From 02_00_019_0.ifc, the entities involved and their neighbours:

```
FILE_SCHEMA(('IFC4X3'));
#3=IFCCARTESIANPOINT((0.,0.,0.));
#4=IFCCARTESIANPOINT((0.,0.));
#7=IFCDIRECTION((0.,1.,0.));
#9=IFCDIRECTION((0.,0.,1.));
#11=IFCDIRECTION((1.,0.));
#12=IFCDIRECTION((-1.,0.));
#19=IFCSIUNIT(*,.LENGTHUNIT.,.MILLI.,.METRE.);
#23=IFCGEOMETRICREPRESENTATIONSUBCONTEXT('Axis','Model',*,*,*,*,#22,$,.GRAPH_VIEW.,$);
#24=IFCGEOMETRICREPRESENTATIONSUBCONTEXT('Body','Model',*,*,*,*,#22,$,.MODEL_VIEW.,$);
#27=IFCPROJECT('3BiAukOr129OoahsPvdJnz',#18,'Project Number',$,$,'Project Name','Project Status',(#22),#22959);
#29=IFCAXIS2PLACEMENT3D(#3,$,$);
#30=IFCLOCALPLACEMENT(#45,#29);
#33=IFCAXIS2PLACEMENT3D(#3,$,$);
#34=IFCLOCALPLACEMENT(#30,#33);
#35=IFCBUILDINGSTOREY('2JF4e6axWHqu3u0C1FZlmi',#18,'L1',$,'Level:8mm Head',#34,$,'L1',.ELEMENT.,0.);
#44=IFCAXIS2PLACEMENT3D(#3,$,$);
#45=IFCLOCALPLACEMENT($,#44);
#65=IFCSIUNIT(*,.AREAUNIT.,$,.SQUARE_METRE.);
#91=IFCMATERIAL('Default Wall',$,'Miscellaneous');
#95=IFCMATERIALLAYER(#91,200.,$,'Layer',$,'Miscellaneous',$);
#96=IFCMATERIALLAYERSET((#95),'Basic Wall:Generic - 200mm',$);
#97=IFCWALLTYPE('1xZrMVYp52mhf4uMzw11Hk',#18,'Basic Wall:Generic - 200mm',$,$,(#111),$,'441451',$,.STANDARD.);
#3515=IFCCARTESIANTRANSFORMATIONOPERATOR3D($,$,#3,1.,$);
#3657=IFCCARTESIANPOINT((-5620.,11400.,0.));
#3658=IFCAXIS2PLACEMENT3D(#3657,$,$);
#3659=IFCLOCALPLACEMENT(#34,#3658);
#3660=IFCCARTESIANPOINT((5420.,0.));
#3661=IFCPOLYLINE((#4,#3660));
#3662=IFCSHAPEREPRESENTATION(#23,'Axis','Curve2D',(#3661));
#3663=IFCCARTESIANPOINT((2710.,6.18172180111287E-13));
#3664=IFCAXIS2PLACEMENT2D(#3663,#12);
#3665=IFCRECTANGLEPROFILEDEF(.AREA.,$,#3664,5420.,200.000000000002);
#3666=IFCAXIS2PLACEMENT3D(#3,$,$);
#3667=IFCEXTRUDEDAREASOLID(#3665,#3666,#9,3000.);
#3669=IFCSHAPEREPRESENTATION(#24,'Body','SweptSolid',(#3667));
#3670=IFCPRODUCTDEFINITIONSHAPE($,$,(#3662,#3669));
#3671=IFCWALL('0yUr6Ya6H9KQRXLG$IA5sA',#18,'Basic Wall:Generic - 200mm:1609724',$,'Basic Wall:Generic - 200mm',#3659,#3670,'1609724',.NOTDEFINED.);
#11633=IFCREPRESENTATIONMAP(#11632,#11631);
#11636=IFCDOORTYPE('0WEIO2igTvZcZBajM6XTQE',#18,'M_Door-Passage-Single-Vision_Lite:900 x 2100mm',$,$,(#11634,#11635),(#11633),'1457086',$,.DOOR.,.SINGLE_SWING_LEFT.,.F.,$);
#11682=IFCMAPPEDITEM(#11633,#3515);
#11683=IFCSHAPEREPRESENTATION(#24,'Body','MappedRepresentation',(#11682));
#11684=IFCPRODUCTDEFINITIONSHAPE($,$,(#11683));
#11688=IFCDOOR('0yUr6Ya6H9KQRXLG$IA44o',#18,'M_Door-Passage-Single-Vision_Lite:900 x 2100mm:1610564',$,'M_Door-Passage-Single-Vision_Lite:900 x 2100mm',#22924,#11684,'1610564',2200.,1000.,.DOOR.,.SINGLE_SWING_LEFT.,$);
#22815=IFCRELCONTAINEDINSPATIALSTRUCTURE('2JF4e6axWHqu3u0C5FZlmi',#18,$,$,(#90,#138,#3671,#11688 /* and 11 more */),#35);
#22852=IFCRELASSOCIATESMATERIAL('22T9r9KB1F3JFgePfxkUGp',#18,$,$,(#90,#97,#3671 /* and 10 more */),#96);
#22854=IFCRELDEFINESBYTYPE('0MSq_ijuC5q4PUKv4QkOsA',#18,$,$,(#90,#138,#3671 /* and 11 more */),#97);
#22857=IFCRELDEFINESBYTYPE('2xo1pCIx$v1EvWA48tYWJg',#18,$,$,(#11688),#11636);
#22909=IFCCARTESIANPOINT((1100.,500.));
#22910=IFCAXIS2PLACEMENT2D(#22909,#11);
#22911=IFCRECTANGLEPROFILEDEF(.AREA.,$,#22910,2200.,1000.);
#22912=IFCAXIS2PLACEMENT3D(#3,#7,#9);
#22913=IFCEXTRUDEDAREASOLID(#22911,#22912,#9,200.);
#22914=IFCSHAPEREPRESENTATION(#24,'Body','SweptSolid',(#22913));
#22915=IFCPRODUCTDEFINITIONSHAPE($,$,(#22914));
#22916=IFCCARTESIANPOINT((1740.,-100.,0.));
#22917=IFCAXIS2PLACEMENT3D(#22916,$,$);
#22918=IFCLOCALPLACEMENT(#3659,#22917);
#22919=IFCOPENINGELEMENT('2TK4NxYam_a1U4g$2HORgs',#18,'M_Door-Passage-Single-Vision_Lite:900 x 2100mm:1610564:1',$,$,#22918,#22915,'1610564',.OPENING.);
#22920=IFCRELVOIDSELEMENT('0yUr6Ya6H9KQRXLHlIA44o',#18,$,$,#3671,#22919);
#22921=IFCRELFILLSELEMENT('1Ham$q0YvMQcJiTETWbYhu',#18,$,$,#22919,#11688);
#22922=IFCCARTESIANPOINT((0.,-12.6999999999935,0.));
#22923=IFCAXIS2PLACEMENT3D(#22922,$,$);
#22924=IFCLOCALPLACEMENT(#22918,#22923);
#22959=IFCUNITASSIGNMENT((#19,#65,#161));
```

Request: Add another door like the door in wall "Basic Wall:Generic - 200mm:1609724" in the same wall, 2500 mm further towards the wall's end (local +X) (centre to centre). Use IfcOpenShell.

```python
import ifcopenshell
import ifcopenshell.api.feature
import ifcopenshell.api.geometry
import ifcopenshell.api.root
import ifcopenshell.geom
import ifcopenshell.util.element
import ifcopenshell.util.placement
import ifcopenshell.util.shape
import ifcopenshell.util.unit

model = ifcopenshell.open("02_00_019_0.ifc")
unit_scale = ifcopenshell.util.unit.calculate_unit_scale(model)
settings = ifcopenshell.geom.settings()


def volume(element):
    """Net volume in cubic metres, openings subtracted."""
    shape = ifcopenshell.geom.create_shape(settings, element)
    return ifcopenshell.util.shape.get_volume(shape.geometry)


def reuse_history(source, copy):
    """copy_class also copies each property set's owner history, people and application; keep the originals."""
    for rel in copy.IsDefinedBy:
        if rel.is_a("IfcRelDefinesByProperties") and (history := rel.RelatingPropertyDefinition.OwnerHistory):
            rel.RelatingPropertyDefinition.OwnerHistory = source.OwnerHistory
            ifcopenshell.util.element.remove_deep2(model, history)


door = model.by_id(11688)
opening = door.FillsVoids[0].RelatingOpeningElement
wall = opening.VoidsElements[0].RelatingBuildingElement
before = volume(wall)
shift = ifcopenshell.util.placement.get_local_placement(wall.ObjectPlacement)[:3, 0] * 2.5 / unit_scale

# copy_class copies the void relationship, type, container and properties, but no geometry.
new_opening = ifcopenshell.api.root.copy_class(model, product=opening)
new_opening.Representation = ifcopenshell.util.element.copy_deep(
    model, opening.Representation, exclude=["IfcGeometricRepresentationContext", "IfcRepresentationMap"]
)
new_opening.Name = "M_Door-Passage-Single-Vision_Lite:900 x 2100mm"
new_opening.Tag = None
new_door = ifcopenshell.api.root.copy_class(model, product=door)
new_door.Representation = ifcopenshell.util.element.copy_deep(
    model, door.Representation, exclude=["IfcGeometricRepresentationContext", "IfcRepresentationMap"]
)
new_door.Name = "M_Door-Passage-Single-Vision_Lite:900 x 2100mm"
new_door.Tag = None
reuse_history(door, new_door)
ifcopenshell.api.feature.add_filling(model, opening=new_opening, element=new_door)

for old, new in ((opening, new_opening), (door, new_door)):
    matrix = ifcopenshell.util.placement.get_local_placement(old.ObjectPlacement)
    matrix[:3, 3] += shift
    ifcopenshell.api.geometry.edit_object_placement(model, product=new, matrix=matrix, is_si=False)

after = volume(wall)

print(f"wall volume {before:.3f} -> {after:.3f} m3")

model.write("02_00_019_0-out.ifc")
```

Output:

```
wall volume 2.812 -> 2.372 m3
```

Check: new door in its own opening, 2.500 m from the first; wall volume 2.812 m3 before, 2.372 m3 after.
